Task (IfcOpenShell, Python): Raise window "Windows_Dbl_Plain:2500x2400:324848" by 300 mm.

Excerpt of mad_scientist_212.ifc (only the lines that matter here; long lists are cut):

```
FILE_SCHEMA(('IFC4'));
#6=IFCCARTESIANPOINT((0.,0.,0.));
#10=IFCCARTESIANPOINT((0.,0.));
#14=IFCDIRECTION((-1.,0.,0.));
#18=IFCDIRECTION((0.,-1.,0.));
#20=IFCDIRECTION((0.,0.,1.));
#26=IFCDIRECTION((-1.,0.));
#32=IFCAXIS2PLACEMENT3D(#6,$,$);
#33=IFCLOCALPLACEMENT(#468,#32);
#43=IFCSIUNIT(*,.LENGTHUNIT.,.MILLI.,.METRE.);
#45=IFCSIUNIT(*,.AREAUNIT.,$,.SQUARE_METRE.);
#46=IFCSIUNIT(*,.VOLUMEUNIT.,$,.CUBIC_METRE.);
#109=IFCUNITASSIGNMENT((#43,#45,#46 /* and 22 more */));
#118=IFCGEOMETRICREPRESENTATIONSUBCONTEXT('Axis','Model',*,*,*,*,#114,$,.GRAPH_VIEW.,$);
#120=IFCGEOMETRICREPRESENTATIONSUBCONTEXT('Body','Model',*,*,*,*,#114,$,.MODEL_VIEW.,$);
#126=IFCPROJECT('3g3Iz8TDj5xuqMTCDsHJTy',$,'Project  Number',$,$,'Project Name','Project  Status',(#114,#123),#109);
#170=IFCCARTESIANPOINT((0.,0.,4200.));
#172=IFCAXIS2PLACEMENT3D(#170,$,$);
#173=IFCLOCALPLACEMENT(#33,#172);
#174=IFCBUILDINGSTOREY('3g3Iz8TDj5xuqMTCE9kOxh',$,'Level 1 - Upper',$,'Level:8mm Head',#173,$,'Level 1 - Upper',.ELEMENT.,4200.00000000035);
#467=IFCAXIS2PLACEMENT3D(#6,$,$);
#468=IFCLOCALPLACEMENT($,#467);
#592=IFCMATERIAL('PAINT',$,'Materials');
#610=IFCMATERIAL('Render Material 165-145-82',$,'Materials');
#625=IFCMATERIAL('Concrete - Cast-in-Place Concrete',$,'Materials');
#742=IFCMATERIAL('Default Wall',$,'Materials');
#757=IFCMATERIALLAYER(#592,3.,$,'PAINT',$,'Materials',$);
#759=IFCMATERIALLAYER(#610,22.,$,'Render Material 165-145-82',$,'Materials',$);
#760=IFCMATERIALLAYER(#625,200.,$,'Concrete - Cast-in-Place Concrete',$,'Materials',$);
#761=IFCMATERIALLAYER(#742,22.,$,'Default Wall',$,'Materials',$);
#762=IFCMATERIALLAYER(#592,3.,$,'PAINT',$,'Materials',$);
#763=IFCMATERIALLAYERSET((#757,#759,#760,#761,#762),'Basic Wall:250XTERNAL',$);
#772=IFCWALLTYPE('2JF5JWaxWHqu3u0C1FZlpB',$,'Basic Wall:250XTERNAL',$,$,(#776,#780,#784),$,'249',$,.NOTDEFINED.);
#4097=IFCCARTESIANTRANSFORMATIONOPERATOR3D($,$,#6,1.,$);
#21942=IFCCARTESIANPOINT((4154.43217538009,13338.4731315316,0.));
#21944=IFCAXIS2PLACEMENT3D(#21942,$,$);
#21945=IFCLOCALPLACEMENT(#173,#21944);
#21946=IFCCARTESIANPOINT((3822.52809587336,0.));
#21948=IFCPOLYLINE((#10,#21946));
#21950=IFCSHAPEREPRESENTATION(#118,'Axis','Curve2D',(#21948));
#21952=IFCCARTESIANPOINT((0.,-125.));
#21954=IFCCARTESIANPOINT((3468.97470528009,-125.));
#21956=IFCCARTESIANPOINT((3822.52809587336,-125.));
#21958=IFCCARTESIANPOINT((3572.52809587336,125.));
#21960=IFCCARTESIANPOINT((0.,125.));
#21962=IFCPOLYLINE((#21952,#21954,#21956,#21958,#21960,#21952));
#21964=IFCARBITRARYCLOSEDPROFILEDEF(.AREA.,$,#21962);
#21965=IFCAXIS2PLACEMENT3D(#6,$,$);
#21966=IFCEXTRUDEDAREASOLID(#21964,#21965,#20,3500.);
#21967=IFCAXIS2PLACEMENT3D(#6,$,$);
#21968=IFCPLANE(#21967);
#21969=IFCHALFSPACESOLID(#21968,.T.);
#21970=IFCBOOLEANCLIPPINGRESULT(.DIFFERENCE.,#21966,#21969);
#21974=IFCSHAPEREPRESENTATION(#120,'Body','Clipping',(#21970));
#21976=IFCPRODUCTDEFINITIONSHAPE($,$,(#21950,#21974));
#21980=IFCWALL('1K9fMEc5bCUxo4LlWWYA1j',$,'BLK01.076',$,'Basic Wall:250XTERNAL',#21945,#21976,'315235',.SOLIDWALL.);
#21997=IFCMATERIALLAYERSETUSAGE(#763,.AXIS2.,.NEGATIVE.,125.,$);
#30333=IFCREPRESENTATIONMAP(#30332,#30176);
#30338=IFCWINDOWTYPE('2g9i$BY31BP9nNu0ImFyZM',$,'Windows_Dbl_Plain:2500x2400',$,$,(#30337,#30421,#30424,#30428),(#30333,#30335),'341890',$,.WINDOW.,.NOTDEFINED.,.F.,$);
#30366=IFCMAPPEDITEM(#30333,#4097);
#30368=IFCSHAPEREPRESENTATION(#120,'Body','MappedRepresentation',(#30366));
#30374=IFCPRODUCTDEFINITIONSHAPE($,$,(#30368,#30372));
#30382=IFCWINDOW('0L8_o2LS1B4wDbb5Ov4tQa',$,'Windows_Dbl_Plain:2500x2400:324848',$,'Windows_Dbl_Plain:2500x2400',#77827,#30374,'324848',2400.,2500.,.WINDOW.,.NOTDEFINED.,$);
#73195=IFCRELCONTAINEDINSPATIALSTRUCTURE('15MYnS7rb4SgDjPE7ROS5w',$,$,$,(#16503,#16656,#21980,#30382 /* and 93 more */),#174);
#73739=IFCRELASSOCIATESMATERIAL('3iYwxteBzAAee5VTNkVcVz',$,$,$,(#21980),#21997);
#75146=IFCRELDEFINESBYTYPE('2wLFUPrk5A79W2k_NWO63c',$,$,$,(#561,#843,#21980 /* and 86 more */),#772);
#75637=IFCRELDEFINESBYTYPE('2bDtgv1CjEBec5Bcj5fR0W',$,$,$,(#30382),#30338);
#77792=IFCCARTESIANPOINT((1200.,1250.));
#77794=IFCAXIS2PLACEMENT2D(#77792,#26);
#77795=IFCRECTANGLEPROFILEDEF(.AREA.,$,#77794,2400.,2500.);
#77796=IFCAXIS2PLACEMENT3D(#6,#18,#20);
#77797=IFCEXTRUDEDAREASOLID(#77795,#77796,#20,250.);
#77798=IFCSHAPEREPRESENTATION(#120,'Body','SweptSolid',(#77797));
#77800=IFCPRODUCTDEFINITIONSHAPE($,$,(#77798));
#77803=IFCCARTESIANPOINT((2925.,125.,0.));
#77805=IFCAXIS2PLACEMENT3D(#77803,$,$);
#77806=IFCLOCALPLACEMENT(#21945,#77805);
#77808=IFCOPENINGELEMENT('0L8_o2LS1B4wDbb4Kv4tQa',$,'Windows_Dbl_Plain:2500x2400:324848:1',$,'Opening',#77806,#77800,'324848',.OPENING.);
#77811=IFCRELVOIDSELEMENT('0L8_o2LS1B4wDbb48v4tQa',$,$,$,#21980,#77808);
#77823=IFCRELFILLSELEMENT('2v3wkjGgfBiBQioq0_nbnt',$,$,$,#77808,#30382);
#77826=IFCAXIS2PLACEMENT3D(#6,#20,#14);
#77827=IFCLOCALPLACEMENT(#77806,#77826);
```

```python
import numpy as np
import ifcopenshell
import ifcopenshell.api.geometry
import ifcopenshell.util.placement
import ifcopenshell.util.unit

model = ifcopenshell.open("mad_scientist_212.ifc")
unit_scale = ifcopenshell.util.unit.calculate_unit_scale(model)

window = model.by_guid("0L8_o2LS1B4wDbb5Ov4tQa")
opening = window.FillsVoids[0].RelatingOpeningElement
dz = 300.0

shift = np.array([0.0, 0.0, dz])
# The window is placed relative to its opening, so it follows when the opening moves.
matrix = ifcopenshell.util.placement.get_local_placement(opening.ObjectPlacement)
matrix[:3, 3] += shift
ifcopenshell.api.geometry.edit_object_placement(
    model, product=opening, matrix=matrix, is_si=False, should_transform_children=True
)

print(f"moved by {dz * unit_scale:+.3f} m")

model.write("mad_scientist_212_v2.ifc")
```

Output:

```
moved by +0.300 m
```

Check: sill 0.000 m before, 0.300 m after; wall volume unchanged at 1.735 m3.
